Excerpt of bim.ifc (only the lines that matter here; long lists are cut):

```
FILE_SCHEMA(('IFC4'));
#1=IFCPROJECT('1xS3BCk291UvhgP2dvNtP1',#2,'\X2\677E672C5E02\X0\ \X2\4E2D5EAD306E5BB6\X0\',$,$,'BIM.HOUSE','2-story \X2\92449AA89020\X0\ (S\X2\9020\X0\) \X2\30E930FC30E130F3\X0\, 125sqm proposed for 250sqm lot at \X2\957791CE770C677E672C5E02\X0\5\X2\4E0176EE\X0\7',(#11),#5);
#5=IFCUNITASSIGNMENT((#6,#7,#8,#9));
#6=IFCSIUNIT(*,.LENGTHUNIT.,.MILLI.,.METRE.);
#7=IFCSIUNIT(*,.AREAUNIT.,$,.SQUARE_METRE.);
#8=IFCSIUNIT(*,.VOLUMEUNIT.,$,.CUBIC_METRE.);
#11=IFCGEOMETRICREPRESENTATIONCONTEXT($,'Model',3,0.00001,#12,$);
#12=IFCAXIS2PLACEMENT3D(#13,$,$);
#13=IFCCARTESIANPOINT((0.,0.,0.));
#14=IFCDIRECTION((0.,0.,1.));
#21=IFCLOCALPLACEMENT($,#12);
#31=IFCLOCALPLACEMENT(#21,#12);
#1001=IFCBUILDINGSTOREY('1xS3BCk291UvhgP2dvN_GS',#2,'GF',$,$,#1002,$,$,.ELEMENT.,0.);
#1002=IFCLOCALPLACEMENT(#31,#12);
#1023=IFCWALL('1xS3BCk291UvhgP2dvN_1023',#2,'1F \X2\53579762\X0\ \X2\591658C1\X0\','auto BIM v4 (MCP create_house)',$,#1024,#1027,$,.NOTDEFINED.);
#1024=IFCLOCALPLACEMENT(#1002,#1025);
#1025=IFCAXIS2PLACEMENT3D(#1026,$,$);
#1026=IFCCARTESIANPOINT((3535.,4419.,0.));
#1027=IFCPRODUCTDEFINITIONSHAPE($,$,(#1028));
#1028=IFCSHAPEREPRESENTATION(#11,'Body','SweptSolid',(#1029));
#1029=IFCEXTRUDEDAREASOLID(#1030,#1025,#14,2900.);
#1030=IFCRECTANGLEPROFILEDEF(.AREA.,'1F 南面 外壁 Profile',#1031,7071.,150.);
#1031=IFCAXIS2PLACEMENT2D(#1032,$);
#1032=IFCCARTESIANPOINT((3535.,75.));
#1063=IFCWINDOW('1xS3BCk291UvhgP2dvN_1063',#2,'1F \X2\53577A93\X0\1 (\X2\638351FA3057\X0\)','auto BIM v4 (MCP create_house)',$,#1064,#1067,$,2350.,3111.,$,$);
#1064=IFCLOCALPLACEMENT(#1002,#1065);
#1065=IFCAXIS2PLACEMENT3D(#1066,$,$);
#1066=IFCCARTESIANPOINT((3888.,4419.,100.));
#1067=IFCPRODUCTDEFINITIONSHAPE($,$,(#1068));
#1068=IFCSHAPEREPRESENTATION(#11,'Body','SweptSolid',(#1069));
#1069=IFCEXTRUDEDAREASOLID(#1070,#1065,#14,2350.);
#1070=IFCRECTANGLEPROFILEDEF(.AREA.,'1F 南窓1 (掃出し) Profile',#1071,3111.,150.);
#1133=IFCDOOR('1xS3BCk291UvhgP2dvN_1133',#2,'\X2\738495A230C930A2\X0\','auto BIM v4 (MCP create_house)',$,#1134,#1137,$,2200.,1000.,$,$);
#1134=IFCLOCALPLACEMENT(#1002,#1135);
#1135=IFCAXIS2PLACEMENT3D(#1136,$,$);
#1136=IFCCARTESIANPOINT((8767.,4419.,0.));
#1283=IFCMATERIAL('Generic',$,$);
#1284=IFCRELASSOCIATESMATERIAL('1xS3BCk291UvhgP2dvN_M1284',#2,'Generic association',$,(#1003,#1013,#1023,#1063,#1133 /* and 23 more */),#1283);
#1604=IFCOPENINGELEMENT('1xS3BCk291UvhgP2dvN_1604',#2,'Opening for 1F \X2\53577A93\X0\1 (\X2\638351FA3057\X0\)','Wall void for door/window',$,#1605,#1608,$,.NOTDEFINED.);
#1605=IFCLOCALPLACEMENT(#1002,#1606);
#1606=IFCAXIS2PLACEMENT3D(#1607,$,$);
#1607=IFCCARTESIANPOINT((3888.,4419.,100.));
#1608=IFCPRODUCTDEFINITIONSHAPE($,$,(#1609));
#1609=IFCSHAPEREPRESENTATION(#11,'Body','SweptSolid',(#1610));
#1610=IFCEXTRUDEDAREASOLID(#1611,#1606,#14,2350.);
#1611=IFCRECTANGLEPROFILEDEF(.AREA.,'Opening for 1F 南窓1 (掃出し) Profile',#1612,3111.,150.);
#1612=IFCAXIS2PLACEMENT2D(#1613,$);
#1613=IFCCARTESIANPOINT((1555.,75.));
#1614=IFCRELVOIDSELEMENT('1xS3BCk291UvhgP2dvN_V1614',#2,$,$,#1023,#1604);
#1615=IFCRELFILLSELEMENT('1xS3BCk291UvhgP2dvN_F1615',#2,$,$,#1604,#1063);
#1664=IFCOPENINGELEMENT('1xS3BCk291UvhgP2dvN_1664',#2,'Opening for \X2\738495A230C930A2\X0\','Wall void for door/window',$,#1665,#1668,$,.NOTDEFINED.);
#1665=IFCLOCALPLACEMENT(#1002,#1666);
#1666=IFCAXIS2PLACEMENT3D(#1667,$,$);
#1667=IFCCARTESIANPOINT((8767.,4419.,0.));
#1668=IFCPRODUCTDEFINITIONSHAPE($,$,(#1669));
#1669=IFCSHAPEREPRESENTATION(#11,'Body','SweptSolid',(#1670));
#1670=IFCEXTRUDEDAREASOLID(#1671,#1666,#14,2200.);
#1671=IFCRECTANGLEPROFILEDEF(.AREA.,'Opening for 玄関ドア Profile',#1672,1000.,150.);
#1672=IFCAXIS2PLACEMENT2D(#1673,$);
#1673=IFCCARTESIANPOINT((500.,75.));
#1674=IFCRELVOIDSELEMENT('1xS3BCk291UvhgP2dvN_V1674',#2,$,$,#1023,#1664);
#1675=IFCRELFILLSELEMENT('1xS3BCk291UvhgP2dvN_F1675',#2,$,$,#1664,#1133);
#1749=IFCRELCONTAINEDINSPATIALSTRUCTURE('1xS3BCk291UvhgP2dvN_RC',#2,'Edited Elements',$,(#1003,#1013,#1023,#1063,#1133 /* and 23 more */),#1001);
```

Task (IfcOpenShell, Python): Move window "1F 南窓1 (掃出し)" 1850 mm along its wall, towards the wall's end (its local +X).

```python
import ifcopenshell
import ifcopenshell.api.geometry
import ifcopenshell.util.placement
import ifcopenshell.util.unit

model = ifcopenshell.open("bim.ifc")
unit_scale = ifcopenshell.util.unit.calculate_unit_scale(model)

window = model.by_guid("1xS3BCk291UvhgP2dvN_1063")
opening = window.FillsVoids[0].RelatingOpeningElement
wall = opening.VoidsElements[0].RelatingBuildingElement

wall_matrix = ifcopenshell.util.placement.get_local_placement(wall.ObjectPlacement)
shift = wall_matrix[:3, 0] * 1.85 / unit_scale
before = ifcopenshell.util.placement.get_local_placement(window.ObjectPlacement)[:3, 3].copy()

# The window is not placed relative to its opening, so move both.
for product in (opening, window):
    matrix = ifcopenshell.util.placement.get_local_placement(product.ObjectPlacement)
    matrix[:3, 3] += shift
    ifcopenshell.api.geometry.edit_object_placement(model, product=product, matrix=matrix, is_si=False)

after = ifcopenshell.util.placement.get_local_placement(window.ObjectPlacement)[:3, 3]
print("window moved by", (after - before).round(3) + 0.0)

model.write("bim-out.ifc")
```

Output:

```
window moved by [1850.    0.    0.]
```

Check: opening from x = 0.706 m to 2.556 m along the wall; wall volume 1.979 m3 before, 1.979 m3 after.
